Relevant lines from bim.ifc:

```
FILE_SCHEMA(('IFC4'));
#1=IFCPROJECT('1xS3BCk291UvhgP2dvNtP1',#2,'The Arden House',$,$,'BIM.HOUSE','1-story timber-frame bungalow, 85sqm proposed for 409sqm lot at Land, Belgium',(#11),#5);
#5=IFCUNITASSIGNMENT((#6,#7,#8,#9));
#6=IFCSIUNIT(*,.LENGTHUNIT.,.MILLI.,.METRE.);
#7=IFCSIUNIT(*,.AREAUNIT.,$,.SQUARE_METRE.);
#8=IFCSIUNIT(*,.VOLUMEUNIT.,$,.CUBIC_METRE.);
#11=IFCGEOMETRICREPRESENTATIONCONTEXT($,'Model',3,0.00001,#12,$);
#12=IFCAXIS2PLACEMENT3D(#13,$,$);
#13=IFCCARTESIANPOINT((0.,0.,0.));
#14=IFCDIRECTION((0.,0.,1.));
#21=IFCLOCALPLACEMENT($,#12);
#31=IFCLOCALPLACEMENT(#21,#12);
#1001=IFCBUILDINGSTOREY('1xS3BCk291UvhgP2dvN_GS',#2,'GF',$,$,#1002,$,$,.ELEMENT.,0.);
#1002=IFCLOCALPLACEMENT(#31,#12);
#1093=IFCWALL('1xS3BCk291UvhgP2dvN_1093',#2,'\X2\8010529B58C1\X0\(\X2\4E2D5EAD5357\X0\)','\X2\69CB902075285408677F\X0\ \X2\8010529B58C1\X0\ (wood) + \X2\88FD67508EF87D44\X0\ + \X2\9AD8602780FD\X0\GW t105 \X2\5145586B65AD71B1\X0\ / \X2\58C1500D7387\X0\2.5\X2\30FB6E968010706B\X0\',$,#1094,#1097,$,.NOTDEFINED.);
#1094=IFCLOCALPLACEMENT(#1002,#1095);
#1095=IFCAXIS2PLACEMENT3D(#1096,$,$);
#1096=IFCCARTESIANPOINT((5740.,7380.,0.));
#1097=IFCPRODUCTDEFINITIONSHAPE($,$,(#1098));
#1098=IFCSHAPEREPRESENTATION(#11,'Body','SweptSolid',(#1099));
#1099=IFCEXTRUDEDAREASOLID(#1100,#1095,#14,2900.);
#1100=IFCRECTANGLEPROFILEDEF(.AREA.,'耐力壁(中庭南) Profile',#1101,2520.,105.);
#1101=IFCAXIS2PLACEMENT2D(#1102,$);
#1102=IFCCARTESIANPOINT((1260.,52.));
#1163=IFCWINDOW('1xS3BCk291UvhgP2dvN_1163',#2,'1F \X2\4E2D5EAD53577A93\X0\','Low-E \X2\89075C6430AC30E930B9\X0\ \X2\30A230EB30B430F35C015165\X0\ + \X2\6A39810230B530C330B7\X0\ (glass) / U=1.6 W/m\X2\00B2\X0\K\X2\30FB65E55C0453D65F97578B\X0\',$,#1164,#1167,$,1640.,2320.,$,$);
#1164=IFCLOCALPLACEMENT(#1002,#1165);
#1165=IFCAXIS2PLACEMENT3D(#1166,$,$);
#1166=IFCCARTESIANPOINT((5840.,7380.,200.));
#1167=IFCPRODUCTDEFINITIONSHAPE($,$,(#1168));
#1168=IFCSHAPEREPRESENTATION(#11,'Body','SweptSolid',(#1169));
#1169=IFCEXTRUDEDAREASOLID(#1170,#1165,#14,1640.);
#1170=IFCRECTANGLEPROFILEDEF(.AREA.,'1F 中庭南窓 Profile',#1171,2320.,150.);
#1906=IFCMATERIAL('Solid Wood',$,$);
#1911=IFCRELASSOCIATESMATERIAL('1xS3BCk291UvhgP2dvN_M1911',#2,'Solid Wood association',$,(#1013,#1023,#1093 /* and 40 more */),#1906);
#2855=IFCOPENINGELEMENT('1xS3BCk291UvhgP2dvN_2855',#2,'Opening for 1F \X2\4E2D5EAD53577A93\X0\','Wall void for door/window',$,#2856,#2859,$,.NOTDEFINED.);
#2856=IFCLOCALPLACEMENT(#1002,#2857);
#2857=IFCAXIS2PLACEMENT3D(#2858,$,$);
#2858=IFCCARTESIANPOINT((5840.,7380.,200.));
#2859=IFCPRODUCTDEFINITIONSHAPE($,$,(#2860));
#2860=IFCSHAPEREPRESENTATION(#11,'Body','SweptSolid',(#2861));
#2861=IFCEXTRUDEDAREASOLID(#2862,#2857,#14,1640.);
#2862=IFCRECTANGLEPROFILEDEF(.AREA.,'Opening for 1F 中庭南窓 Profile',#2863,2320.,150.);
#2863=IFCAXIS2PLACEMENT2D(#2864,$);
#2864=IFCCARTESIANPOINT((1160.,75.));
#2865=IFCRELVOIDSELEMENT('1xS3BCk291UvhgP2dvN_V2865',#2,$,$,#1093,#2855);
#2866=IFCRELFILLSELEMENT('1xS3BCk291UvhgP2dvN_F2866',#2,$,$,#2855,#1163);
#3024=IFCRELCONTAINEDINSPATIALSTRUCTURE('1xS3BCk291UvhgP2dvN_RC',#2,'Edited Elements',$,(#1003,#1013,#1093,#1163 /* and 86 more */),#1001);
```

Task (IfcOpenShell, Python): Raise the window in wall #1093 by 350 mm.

```python
import numpy as np
import ifcopenshell
import ifcopenshell.api.geometry
import ifcopenshell.util.placement
import ifcopenshell.util.unit

model = ifcopenshell.open("bim.ifc")
unit_scale = ifcopenshell.util.unit.calculate_unit_scale(model)

window = model.by_id(1163)
opening = window.FillsVoids[0].RelatingOpeningElement
dz = 0.35 / unit_scale

shift = np.array([0.0, 0.0, dz])
# The window is not placed relative to its opening, so move both.
for product in (opening, window):
    matrix = ifcopenshell.util.placement.get_local_placement(product.ObjectPlacement)
    matrix[:3, 3] += shift
    ifcopenshell.api.geometry.edit_object_placement(model, product=product, matrix=matrix, is_si=False)

print(f"moved by {dz * unit_scale:+.3f} m")

model.write("bim-out.ifc")
```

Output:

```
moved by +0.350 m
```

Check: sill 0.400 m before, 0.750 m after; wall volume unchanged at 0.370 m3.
